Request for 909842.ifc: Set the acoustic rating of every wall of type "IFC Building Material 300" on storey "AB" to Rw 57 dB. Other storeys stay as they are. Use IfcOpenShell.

First a look at what the model holds.

```python
import ifcopenshell
import ifcopenshell.util.element

model = ifcopenshell.open("909842.ifc")
print(model.schema)
storey = next(s for s in model.by_type("IfcBuildingStorey") if s.Name == "AB")
walls = [e for e in ifcopenshell.util.element.get_decomposition(storey) if e.is_a("IfcWall")]
seen = {}
for e in walls:
    element_type = ifcopenshell.util.element.get_type(e)
    key = (element_type.Name if element_type != e and element_type else None, ifcopenshell.util.element.get_pset(e, "Pset_WallCommon", "AcousticRating"))
    seen[key] = seen.get(key, 0) + 1
for (name, value), count in sorted(seen.items(), key=str):
    print(count, "x", name, "|", value)
```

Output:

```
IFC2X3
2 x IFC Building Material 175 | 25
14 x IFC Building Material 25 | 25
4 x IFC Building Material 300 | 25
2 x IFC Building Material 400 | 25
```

```python
import ifcopenshell
import ifcopenshell.api.pset
import ifcopenshell.util.element

model = ifcopenshell.open("909842.ifc")

storey = next(s for s in model.by_type("IfcBuildingStorey") if s.Name == "AB")
walls = [e for e in ifcopenshell.util.element.get_decomposition(storey) if e.is_a("IfcWall")]

count = 0
for e in walls:
    element_type = ifcopenshell.util.element.get_type(e)
    if element_type in (None, e) or element_type.Name != "IFC Building Material 300":
        continue
    # add_pset returns the element's existing set when there is one.
    pset = ifcopenshell.api.pset.add_pset(model, product=e, name="Pset_WallCommon")
    ifcopenshell.api.pset.edit_pset(model, pset=pset, properties={"AcousticRating": "Rw 57 dB"})
    count += 1

print(count, "walls updated")

model.write("909842_edited.ifc")
```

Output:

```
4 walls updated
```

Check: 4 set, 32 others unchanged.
